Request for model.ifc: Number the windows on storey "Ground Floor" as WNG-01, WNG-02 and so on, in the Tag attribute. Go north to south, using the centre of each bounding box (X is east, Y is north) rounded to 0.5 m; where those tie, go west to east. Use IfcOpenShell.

First a look at what the model holds.

```python
import ifcopenshell
import ifcopenshell.util.element
import ifcopenshell.util.placement

model = ifcopenshell.open("model.ifc")
print(model.schema)
storey = next(s for s in model.by_type("IfcBuildingStorey") if s.Name == "Ground Floor")
windows = [e for e in ifcopenshell.util.element.get_decomposition(storey) if e.is_a("IfcWindow")]
for e in sorted(windows, key=lambda e: e.id()):
    origin = ifcopenshell.util.placement.get_local_placement(e.ObjectPlacement)[:3, 3]
    print(e.id(), e.Tag, e.Name, origin.round(2) + 0.0, sep=" | ")
```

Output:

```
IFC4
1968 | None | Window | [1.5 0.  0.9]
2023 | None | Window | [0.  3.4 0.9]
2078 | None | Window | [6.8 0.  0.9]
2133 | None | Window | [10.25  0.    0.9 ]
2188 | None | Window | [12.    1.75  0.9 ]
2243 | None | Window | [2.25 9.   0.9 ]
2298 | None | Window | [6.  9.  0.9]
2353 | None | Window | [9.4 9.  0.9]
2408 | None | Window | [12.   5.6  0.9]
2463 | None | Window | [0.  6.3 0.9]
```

```python
import ifcopenshell
import ifcopenshell.geom
import ifcopenshell.util.element
import ifcopenshell.util.shape

model = ifcopenshell.open("model.ifc")
settings = ifcopenshell.geom.settings()
settings.set("use-world-coords", True)


def centre(element):
    shape = ifcopenshell.geom.create_shape(settings, element)
    return ifcopenshell.util.shape.get_bbox_centroid(shape.geometry)


storey = next(s for s in model.by_type("IfcBuildingStorey") if s.Name == "Ground Floor")
windows = [e for e in ifcopenshell.util.element.get_decomposition(storey) if e.is_a("IfcWindow")]

# Insertion points can sit at a corner or the storey origin, so sort by the geometry (in metres).
centres = {e: centre(e) for e in windows}
windows.sort(key=lambda e: (-round(centres[e][1] / 0.5), centres[e][0]))

for i, e in enumerate(windows, start=1):
    number = f"WNG-{i:02d}"
    e.Tag = number
    print(e.id(), number)

model.write("model_edited.ifc")
```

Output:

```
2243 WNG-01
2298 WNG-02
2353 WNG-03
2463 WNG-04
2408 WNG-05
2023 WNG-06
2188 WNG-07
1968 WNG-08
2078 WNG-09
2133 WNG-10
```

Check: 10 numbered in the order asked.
